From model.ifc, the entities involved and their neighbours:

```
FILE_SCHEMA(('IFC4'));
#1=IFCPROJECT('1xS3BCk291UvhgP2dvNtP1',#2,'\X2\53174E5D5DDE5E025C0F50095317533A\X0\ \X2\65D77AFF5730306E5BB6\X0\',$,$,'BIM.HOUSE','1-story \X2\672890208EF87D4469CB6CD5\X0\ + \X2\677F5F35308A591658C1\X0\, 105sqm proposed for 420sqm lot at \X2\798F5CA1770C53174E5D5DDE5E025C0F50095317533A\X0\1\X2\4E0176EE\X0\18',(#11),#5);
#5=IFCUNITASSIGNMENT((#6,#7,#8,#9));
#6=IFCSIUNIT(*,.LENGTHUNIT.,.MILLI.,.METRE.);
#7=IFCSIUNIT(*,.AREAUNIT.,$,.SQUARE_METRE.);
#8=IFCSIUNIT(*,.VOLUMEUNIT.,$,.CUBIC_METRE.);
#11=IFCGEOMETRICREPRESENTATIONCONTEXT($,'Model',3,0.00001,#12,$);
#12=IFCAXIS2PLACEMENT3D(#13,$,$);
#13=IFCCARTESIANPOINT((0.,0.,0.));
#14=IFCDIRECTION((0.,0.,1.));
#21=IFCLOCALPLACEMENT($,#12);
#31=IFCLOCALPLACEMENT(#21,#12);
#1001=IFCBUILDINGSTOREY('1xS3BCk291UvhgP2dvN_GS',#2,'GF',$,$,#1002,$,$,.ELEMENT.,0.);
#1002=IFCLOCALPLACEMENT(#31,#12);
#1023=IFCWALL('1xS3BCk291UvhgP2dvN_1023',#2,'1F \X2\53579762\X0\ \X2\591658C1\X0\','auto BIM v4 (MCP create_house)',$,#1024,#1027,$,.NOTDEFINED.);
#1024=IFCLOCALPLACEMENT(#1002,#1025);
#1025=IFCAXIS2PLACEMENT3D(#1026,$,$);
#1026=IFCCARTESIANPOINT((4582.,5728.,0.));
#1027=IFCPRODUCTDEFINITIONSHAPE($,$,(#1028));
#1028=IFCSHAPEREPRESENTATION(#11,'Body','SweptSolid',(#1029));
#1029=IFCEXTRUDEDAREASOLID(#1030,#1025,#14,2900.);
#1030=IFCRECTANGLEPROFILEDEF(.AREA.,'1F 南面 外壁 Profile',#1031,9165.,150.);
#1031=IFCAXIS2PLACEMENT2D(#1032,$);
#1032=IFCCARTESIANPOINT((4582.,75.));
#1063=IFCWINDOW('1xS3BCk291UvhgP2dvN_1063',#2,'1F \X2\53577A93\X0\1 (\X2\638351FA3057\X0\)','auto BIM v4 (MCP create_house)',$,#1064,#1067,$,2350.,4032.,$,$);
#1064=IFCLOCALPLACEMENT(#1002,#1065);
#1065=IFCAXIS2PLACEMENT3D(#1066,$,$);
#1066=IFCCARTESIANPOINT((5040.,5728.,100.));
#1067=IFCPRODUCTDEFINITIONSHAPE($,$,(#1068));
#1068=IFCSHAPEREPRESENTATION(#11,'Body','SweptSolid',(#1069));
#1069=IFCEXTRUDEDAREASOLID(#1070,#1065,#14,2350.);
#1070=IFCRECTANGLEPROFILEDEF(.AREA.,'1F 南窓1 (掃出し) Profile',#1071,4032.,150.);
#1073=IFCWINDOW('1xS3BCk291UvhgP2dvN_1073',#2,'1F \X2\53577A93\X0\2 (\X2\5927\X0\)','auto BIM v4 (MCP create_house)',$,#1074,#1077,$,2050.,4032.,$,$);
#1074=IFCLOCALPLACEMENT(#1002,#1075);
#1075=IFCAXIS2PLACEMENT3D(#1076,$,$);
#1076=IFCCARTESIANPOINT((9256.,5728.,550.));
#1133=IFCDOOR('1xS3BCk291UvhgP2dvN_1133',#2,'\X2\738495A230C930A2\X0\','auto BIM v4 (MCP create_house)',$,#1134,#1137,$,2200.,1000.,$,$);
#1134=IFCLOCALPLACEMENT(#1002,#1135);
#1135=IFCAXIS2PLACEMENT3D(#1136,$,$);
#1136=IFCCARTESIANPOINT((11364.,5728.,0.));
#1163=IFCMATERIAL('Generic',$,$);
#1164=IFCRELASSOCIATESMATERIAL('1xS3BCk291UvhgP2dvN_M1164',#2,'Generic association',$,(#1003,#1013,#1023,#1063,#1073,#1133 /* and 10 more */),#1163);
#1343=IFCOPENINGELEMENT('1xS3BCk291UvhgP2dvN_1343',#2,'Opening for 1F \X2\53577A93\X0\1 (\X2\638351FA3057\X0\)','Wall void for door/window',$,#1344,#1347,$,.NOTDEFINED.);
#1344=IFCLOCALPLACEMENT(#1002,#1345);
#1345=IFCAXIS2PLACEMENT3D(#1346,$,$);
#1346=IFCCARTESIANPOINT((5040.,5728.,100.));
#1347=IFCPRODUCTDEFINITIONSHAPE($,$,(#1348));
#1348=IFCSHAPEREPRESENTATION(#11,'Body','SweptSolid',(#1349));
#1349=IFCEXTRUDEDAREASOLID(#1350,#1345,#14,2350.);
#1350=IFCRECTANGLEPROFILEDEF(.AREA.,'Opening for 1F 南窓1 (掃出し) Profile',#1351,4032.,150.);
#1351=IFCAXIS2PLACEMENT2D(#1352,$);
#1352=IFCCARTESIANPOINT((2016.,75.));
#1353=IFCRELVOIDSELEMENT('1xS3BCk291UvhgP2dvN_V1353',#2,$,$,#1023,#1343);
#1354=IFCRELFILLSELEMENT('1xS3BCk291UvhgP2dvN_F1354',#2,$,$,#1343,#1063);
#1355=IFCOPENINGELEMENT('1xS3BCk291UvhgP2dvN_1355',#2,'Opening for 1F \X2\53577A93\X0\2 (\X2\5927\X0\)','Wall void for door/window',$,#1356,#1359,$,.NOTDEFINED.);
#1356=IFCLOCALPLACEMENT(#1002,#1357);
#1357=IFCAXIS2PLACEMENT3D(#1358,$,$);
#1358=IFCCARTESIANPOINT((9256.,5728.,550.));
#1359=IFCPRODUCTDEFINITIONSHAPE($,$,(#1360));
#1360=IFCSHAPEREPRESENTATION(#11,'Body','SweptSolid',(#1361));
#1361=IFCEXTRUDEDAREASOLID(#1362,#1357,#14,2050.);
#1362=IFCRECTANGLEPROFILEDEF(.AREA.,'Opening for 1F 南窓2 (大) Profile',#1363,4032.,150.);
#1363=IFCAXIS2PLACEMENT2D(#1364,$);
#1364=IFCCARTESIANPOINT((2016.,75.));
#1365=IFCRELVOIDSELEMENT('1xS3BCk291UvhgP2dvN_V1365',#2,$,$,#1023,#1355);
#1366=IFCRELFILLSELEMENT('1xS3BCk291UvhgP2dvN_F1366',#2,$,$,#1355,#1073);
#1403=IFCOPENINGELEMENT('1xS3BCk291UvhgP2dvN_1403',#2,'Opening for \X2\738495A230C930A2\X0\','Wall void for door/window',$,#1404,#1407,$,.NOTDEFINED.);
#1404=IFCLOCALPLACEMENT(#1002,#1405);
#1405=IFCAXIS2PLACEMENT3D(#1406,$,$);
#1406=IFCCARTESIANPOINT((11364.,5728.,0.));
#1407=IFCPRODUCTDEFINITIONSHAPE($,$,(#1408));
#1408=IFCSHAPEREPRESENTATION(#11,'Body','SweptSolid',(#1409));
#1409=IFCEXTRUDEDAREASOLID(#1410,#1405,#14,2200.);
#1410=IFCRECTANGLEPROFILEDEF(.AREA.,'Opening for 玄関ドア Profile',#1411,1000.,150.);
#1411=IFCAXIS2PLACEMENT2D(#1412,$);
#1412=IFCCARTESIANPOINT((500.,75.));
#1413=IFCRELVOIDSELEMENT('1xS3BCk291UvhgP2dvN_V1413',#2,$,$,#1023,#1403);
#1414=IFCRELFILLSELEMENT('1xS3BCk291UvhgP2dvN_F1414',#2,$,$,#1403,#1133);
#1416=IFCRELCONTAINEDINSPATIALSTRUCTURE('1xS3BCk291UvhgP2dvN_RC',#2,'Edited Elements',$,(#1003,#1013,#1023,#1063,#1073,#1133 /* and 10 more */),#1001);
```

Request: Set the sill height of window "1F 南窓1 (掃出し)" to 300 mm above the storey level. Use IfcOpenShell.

```python
import numpy as np
import ifcopenshell
import ifcopenshell.api.geometry
import ifcopenshell.geom
import ifcopenshell.util.element
import ifcopenshell.util.placement
import ifcopenshell.util.shape
import ifcopenshell.util.unit

model = ifcopenshell.open("model.ifc")
unit_scale = ifcopenshell.util.unit.calculate_unit_scale(model)

window = model.by_id(1063)
opening = window.FillsVoids[0].RelatingOpeningElement
storey = ifcopenshell.util.element.get_container(window, ifc_class="IfcBuildingStorey")
level = ifcopenshell.util.placement.get_local_placement(storey.ObjectPlacement)[2, 3]

# The opening's origin need not be at the sill, so measure its lowest point.
shape = ifcopenshell.geom.create_shape(ifcopenshell.geom.settings(), opening)
bottom = ifcopenshell.util.shape.get_shape_bottom_elevation(shape, shape.geometry) / unit_scale
dz = level + 300.0 - bottom

shift = np.array([0.0, 0.0, dz])
# The window is not placed relative to its opening, so move both.
for product in (opening, window):
    matrix = ifcopenshell.util.placement.get_local_placement(product.ObjectPlacement)
    matrix[:3, 3] += shift
    ifcopenshell.api.geometry.edit_object_placement(model, product=product, matrix=matrix, is_si=False)

print(f"moved by {dz * unit_scale:+.3f} m")

model.write("model-out.ifc")
```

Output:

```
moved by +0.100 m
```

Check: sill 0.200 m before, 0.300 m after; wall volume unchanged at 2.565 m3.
